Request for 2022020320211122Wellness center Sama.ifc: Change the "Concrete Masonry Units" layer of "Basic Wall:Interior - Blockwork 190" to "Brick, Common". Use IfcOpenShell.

First a look at what the model holds.

```python
import ifcopenshell
import ifcopenshell.util.element

model = ifcopenshell.open("2022020320211122Wellness center Sama.ifc")
print(model.schema)
for layer_set in model.by_type("IfcMaterialLayerSet"):
    if layer_set.LayerSetName == "Basic Wall:Interior - Blockwork 190":
        for layer in layer_set.MaterialLayers:
            print(layer.id(), layer.Material and layer.Material.Name, layer.LayerThickness, sep=" | ")
        print(len(ifcopenshell.util.element.get_elements_by_material(model, layer_set)), "elements and types use it")
print(sorted(m.Name for m in model.by_type("IfcMaterial") if m.Name)[:60])
```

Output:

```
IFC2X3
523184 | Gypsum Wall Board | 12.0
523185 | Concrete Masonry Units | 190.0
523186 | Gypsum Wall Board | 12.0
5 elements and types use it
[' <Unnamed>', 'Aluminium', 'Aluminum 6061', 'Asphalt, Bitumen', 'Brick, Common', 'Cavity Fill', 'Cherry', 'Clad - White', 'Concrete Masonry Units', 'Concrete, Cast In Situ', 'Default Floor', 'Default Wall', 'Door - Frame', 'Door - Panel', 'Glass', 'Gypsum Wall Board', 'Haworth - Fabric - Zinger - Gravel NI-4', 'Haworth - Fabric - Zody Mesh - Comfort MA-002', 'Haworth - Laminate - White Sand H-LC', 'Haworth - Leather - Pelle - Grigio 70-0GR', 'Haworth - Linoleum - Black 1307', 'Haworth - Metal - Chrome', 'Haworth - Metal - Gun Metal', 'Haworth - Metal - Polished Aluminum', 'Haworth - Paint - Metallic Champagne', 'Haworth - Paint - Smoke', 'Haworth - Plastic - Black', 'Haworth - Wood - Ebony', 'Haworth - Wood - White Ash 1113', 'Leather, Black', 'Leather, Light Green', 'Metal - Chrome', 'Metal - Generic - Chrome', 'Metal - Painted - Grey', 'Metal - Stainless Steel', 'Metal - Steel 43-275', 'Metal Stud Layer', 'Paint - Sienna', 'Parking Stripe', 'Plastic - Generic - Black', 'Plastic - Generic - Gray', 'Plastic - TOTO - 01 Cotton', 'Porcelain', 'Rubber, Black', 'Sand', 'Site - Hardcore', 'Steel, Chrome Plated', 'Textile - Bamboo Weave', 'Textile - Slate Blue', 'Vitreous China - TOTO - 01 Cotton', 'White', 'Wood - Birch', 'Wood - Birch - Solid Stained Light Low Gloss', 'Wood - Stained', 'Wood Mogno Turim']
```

```python
import ifcopenshell
import ifcopenshell.api.material

model = ifcopenshell.open("2022020320211122Wellness center Sama.ifc")

layer_set = next(s for s in model.by_type("IfcMaterialLayerSet") if s.LayerSetName == "Basic Wall:Interior - Blockwork 190")
layer = next(l for l in layer_set.MaterialLayers if l.Material and l.Material.Name == "Concrete Masonry Units")
material = next(m for m in model.by_type("IfcMaterial") if m.Name == "Brick, Common")

# Point this one layer at the other material; renaming the old one would change it everywhere.
ifcopenshell.api.material.edit_layer(model, layer=layer, attributes={}, material=material)

print([l.Material.Name if l.Material else None for l in layer_set.MaterialLayers])

model.write("2022020320211122Wellness center Sama_v2.ifc")
```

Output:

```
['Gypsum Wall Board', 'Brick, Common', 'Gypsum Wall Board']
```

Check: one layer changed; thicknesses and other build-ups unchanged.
